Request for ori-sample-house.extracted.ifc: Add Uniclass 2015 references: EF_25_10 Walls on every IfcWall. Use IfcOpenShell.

First a look at what the model holds.

```python
import ifcopenshell

model = ifcopenshell.open("ori-sample-house.extracted.ifc")
print(model.schema)
print("classifications:", [c.Name for c in model.by_type("IfcClassification")])
for ifc_class in ("IfcDoor", "IfcRoof", "IfcStair", "IfcWall", "IfcWindow"):
    print(ifc_class, len(model.by_type(ifc_class)))
```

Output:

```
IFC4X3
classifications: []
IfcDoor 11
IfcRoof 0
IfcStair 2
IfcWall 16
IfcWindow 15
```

```python
import ifcopenshell
import ifcopenshell.api.classification

model = ifcopenshell.open("ori-sample-house.extracted.ifc")

system = ifcopenshell.api.classification.add_classification(model, classification="Uniclass 2015")

codes = {
    "IfcWall": ("EF_25_10", "Walls"),
}
for ifc_class, (code, name) in codes.items():
    products = model.by_type(ifc_class)
    ifcopenshell.api.classification.add_reference(
        model, products=products, classification=system, identification=code, name=name
    )
    print(code, len(products))

model.write("ori-sample-house.extracted_v2.ifc")
```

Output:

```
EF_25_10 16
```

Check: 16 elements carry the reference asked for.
